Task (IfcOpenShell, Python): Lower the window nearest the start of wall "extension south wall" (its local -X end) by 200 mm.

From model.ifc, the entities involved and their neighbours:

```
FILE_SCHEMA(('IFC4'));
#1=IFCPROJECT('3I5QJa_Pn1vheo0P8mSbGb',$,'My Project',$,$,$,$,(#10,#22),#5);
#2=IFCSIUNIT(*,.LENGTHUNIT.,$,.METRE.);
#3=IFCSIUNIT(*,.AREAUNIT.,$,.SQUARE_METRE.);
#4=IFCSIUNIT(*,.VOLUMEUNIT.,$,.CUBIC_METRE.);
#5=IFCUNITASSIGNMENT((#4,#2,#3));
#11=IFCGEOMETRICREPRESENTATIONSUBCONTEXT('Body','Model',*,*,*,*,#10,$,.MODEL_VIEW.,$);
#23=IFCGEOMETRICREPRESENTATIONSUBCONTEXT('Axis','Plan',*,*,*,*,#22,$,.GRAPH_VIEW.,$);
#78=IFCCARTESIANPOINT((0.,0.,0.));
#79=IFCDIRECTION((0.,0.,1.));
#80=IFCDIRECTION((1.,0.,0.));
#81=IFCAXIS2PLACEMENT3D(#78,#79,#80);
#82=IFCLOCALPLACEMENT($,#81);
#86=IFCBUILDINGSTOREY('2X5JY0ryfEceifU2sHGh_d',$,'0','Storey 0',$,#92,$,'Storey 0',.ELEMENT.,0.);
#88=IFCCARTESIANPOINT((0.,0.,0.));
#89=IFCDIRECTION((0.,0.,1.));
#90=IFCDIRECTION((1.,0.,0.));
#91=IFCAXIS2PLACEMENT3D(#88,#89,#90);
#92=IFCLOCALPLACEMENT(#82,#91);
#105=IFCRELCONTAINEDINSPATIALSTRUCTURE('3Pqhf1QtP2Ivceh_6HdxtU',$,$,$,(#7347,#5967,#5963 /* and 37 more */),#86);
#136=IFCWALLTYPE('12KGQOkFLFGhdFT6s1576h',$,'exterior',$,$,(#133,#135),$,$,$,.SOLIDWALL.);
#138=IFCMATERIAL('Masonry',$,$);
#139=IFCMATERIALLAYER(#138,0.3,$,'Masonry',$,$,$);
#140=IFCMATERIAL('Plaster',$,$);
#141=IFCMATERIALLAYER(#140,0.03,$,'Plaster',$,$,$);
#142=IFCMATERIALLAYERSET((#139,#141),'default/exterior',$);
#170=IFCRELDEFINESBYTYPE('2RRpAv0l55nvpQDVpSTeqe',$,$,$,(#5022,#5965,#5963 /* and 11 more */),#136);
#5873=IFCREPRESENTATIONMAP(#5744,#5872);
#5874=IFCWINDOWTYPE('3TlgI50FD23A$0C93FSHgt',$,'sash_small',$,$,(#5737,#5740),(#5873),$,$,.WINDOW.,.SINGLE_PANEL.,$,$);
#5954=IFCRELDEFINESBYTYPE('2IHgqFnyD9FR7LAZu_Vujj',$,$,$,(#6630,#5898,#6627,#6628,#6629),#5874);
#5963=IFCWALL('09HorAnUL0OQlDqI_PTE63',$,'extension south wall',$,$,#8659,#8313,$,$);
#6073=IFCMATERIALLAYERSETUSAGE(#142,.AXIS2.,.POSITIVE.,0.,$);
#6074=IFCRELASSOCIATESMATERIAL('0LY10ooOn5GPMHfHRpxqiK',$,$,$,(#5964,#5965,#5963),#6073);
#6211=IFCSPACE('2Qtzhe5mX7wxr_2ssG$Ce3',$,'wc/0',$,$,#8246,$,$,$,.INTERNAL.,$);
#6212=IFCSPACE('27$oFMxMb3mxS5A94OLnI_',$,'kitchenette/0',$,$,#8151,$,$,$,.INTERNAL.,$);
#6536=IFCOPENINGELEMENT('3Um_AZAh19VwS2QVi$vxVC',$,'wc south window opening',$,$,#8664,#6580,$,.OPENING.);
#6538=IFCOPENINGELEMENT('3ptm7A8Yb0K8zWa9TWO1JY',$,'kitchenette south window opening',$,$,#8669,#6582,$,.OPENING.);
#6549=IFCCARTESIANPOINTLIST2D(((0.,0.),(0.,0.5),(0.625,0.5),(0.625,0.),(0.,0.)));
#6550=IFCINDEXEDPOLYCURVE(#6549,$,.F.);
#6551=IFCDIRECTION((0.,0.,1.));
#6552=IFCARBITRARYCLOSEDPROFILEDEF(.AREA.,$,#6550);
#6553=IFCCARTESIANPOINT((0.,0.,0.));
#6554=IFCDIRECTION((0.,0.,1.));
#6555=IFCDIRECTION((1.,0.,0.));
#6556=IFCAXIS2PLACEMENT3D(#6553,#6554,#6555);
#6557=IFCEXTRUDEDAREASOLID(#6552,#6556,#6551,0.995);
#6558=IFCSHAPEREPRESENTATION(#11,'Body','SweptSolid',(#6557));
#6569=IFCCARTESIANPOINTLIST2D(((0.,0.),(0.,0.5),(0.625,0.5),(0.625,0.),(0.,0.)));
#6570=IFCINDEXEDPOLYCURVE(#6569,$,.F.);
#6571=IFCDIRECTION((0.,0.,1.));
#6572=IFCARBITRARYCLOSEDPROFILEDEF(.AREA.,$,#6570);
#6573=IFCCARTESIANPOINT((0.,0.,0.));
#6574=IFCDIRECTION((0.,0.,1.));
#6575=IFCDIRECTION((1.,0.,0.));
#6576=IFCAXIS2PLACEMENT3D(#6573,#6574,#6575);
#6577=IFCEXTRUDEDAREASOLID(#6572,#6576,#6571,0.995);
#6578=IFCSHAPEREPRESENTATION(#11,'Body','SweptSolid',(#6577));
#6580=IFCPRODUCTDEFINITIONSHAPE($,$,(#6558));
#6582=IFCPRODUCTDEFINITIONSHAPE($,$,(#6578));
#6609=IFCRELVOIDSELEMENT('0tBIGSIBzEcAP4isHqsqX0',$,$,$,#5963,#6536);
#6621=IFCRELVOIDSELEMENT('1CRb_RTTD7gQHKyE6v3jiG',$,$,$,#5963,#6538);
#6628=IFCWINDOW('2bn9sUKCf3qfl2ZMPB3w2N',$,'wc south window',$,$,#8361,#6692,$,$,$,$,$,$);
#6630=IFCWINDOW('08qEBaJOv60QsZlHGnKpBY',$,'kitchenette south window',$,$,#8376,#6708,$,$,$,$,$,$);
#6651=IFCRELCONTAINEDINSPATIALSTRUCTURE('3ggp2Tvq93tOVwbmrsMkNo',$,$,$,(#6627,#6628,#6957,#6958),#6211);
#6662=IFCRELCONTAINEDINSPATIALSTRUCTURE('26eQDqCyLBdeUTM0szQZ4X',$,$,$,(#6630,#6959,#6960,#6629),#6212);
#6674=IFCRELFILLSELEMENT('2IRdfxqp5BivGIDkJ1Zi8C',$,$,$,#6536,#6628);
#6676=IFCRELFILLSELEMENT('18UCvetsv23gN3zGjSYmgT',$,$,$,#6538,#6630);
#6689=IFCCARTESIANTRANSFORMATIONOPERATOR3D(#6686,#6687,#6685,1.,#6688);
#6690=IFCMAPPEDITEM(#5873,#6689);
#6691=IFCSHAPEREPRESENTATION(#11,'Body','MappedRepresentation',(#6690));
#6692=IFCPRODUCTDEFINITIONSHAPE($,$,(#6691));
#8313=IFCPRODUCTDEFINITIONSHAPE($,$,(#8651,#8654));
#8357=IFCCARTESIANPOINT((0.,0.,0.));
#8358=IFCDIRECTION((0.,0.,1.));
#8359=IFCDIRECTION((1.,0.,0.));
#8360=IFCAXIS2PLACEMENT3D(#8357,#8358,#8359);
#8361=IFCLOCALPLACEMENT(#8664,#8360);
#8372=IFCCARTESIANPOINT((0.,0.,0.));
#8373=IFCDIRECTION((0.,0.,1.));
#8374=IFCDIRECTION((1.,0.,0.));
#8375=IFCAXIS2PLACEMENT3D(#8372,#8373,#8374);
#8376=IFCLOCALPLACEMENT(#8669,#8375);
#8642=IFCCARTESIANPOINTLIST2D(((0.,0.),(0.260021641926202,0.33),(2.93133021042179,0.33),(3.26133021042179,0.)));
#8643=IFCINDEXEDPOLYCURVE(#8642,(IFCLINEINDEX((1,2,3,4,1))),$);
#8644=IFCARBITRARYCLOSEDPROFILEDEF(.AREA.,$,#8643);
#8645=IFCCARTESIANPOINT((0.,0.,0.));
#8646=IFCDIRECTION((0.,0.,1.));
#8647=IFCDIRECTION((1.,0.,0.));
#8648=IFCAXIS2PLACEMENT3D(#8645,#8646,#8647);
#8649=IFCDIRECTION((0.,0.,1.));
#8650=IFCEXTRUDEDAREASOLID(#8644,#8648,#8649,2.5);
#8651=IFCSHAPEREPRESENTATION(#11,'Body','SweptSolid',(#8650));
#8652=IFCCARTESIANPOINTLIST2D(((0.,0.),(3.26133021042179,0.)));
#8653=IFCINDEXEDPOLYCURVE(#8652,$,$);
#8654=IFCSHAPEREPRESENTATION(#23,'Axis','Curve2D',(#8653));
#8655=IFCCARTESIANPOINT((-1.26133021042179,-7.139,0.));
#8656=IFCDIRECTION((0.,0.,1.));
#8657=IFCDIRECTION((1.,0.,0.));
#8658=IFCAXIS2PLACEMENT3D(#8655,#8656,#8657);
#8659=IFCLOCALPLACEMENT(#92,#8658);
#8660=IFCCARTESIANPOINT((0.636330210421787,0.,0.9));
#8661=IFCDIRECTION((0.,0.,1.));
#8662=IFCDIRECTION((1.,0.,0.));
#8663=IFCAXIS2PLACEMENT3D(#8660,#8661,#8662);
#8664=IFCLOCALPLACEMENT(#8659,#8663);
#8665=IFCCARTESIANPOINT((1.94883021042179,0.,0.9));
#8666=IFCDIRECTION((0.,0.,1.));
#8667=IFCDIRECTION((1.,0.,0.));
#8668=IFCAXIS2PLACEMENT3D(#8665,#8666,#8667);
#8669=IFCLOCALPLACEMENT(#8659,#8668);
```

```python
import numpy as np
import ifcopenshell
import ifcopenshell.api.geometry
import ifcopenshell.util.placement
import ifcopenshell.util.unit

model = ifcopenshell.open("model.ifc")
unit_scale = ifcopenshell.util.unit.calculate_unit_scale(model)

window = model.by_guid("2bn9sUKCf3qfl2ZMPB3w2N")
opening = window.FillsVoids[0].RelatingOpeningElement
dz = -0.2

shift = np.array([0.0, 0.0, dz])
# The window is placed relative to its opening, so it follows when the opening moves.
matrix = ifcopenshell.util.placement.get_local_placement(opening.ObjectPlacement)
matrix[:3, 3] += shift
ifcopenshell.api.geometry.edit_object_placement(
    model, product=opening, matrix=matrix, is_si=False, should_transform_children=True
)

print(f"moved by {dz * unit_scale:+.3f} m")

model.write("model_edited.ifc")
```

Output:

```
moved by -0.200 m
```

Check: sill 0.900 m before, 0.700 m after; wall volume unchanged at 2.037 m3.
